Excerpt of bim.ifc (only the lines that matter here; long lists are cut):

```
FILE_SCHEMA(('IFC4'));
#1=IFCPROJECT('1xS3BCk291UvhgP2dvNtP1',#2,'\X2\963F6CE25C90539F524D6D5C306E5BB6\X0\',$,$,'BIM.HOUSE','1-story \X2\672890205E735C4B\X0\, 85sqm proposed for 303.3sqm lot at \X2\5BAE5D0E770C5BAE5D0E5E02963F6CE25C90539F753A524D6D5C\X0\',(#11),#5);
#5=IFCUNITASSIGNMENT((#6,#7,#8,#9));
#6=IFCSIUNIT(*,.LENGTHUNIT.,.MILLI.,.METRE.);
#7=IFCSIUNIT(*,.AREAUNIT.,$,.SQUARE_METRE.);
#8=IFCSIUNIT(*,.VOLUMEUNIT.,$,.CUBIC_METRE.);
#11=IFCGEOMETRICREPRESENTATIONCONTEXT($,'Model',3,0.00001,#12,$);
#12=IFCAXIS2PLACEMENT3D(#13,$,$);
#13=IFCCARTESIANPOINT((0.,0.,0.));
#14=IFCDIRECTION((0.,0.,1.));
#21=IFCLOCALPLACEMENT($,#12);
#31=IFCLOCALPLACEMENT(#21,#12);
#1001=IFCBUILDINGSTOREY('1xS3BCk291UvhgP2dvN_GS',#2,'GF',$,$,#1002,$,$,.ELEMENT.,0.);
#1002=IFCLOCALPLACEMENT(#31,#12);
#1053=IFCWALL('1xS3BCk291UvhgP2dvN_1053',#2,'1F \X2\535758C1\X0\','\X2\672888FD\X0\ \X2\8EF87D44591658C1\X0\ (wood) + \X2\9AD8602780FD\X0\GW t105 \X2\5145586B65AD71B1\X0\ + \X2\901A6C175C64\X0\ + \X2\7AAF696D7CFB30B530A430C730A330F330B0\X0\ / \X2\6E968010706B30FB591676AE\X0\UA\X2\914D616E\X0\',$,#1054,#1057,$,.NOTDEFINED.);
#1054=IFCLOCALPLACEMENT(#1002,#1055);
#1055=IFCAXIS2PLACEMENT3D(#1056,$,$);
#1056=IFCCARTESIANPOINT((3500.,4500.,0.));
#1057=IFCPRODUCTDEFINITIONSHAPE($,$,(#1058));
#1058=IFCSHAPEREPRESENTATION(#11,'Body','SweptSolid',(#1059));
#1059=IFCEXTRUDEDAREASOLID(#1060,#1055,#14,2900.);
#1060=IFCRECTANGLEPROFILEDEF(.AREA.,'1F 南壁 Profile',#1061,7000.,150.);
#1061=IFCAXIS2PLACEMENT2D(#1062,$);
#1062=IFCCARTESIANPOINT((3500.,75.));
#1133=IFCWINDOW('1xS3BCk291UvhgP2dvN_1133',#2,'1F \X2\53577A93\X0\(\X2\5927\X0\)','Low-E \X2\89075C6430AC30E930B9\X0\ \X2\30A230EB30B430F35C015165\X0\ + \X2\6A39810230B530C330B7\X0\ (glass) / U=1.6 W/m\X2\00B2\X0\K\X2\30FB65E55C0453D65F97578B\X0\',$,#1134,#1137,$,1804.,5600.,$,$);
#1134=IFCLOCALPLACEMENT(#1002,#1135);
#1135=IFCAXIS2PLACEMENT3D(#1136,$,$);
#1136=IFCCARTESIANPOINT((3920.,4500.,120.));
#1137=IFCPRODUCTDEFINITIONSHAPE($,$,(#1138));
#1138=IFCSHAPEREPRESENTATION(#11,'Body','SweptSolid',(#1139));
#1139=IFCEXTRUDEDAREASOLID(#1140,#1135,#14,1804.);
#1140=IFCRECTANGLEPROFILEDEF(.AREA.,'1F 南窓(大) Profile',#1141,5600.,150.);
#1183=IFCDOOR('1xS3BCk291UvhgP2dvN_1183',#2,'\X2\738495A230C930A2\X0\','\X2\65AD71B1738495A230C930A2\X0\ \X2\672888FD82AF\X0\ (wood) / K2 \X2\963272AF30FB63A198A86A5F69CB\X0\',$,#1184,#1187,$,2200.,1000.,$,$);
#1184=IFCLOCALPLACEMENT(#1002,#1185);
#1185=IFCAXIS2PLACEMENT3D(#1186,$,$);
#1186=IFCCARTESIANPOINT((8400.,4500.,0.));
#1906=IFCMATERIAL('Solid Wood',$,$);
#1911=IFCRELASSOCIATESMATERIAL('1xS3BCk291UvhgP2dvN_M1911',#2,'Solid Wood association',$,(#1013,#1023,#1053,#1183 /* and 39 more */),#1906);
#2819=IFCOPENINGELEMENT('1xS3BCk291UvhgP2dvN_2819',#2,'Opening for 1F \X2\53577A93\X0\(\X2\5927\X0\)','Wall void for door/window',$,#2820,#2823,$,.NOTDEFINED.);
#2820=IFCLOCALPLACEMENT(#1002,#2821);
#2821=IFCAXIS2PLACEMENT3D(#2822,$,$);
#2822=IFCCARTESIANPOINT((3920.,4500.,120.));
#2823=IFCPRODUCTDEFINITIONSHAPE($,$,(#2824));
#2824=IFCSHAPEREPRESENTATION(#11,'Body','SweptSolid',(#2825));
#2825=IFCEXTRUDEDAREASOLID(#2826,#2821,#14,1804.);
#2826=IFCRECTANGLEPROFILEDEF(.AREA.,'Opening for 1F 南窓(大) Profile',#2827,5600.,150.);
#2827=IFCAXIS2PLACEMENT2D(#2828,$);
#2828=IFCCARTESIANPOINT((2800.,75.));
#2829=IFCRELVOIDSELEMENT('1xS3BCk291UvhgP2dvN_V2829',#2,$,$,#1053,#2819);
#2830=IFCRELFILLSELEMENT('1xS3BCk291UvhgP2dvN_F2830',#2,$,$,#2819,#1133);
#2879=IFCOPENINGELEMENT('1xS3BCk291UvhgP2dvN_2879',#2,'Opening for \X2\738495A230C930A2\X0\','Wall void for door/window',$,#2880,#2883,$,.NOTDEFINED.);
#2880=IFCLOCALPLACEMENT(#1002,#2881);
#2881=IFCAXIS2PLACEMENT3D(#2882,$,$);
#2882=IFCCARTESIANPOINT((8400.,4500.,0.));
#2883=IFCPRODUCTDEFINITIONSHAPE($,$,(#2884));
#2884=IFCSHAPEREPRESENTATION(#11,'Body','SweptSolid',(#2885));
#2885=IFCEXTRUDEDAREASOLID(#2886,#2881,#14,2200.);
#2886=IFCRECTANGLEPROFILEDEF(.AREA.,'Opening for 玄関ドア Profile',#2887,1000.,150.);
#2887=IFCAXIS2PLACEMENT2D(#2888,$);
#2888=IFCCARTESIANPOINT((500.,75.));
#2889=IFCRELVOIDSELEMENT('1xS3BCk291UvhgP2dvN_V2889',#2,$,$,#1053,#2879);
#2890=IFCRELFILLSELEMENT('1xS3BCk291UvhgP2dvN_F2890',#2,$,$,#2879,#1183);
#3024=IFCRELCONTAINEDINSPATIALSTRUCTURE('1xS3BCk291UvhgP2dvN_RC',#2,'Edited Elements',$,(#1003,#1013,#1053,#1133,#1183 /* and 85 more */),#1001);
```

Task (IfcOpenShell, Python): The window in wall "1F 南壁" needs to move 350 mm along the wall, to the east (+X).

```python
import ifcopenshell
import ifcopenshell.api.geometry
import ifcopenshell.util.placement
import ifcopenshell.util.unit

model = ifcopenshell.open("bim.ifc")
unit_scale = ifcopenshell.util.unit.calculate_unit_scale(model)

window = model.by_id(1133)
opening = window.FillsVoids[0].RelatingOpeningElement
wall = opening.VoidsElements[0].RelatingBuildingElement

wall_matrix = ifcopenshell.util.placement.get_local_placement(wall.ObjectPlacement)
shift = wall_matrix[:3, 0] * 0.35 / unit_scale
before = ifcopenshell.util.placement.get_local_placement(window.ObjectPlacement)[:3, 3].copy()

# The window is not placed relative to its opening, so move both.
for product in (opening, window):
    matrix = ifcopenshell.util.placement.get_local_placement(product.ObjectPlacement)
    matrix[:3, 3] += shift
    ifcopenshell.api.geometry.edit_object_placement(model, product=product, matrix=matrix, is_si=False)

after = ifcopenshell.util.placement.get_local_placement(window.ObjectPlacement)[:3, 3]
print("window moved by", (after - before).round(3) + 0.0)

model.write("bim_updated.ifc")
```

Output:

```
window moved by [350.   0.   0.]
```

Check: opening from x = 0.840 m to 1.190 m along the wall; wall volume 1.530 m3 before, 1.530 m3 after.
